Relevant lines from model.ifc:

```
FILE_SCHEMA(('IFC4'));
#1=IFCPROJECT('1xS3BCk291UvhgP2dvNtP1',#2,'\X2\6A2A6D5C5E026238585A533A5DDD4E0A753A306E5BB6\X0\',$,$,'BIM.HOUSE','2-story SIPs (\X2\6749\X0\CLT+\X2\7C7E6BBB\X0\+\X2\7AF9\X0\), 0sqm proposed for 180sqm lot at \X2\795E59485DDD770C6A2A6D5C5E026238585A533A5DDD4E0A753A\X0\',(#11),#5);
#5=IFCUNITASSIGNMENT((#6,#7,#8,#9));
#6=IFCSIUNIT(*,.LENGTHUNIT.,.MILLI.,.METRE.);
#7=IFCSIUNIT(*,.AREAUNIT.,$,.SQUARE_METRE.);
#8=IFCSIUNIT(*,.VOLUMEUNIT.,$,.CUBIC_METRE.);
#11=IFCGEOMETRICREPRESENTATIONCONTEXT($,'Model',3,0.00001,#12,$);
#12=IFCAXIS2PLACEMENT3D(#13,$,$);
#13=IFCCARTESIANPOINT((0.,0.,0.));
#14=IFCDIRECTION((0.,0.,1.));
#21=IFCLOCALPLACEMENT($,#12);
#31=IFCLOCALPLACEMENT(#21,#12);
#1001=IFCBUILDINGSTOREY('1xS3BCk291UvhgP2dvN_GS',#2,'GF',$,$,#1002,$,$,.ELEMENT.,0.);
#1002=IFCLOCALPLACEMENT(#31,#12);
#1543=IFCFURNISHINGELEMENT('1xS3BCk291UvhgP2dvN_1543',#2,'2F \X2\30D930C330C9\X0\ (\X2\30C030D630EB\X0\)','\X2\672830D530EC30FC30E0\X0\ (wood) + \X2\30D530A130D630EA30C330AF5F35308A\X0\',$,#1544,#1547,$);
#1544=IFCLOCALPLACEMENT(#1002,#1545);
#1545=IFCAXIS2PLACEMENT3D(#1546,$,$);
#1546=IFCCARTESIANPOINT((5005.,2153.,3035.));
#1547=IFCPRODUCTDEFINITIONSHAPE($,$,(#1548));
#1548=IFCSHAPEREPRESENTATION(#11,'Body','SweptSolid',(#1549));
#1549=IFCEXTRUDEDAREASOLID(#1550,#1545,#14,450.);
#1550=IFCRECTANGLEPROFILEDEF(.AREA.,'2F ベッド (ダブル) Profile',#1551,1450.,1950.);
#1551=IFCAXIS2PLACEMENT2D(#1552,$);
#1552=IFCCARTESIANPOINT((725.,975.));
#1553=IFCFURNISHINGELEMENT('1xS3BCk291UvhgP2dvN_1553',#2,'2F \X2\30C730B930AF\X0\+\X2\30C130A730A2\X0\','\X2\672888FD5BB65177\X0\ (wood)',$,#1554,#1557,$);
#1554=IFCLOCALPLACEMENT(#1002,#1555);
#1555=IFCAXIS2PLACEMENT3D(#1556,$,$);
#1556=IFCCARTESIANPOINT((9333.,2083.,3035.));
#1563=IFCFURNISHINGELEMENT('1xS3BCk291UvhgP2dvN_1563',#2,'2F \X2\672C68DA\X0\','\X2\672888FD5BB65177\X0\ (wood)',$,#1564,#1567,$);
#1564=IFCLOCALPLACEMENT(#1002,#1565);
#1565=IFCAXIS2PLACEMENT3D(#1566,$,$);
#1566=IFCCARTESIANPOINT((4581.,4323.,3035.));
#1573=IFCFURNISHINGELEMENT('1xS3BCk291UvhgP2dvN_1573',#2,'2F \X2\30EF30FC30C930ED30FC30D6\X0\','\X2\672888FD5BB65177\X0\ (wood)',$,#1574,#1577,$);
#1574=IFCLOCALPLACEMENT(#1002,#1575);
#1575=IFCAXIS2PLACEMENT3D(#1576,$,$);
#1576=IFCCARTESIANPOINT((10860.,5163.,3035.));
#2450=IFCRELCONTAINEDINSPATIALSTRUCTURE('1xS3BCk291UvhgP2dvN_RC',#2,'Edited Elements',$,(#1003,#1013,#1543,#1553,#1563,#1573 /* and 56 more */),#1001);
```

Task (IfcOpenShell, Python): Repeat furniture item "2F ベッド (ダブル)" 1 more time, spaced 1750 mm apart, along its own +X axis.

```python
import ifcopenshell
import ifcopenshell.api.geometry
import ifcopenshell.api.root
import ifcopenshell.util.element
import ifcopenshell.util.placement
import ifcopenshell.util.unit

model = ifcopenshell.open("model.ifc")
unit_scale = ifcopenshell.util.unit.calculate_unit_scale(model)


def reuse_history(source, copy):
    """copy_class also copies each property set's owner history, people and application; keep the originals."""
    for rel in copy.IsDefinedBy:
        if rel.is_a("IfcRelDefinesByProperties") and (history := rel.RelatingPropertyDefinition.OwnerHistory):
            rel.RelatingPropertyDefinition.OwnerHistory = source.OwnerHistory
            ifcopenshell.util.element.remove_deep2(model, history)


source = model.by_id(1543)
base = ifcopenshell.util.placement.get_local_placement(source.ObjectPlacement)
step = base[:3, 0] * 1.75 / unit_scale

for i in range(1, 2):
    copy = ifcopenshell.api.root.copy_class(model, product=source)
    copy.Representation = ifcopenshell.util.element.copy_deep(
        model, source.Representation, exclude=["IfcGeometricRepresentationContext", "IfcRepresentationMap"]
    )
    reuse_history(source, copy)
    matrix = base.copy()
    matrix[:3, 3] += i * step
    print("added at", matrix[:3, 3].round(3) + 0.0)
    ifcopenshell.api.geometry.edit_object_placement(model, product=copy, matrix=matrix, is_si=False)

model.write("model_rev.ifc")
```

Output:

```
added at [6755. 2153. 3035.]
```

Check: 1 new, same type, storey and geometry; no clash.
